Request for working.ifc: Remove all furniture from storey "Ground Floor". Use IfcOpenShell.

First a look at what the model holds.

```python
import ifcopenshell
import ifcopenshell.util.element

model = ifcopenshell.open("working.ifc")
print(model.schema)
storey = next(s for s in model.by_type("IfcBuildingStorey") if s.Name == "Ground Floor")
furniture = [e for e in ifcopenshell.util.element.get_decomposition(storey) if e.is_a("IfcFurnishingElement")]
seen = {}
for e in furniture:
    element_type = ifcopenshell.util.element.get_type(e)
    name = element_type.Name if element_type not in (None, e) else None
    seen[name] = seen.get(name, 0) + 1
for name, count in sorted(seen.items(), key=str):
    print(count, "x", name)
```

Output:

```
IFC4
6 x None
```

```python
import ifcopenshell
import ifcopenshell.api.root
import ifcopenshell.util.element

model = ifcopenshell.open("working.ifc")

storey = next(s for s in model.by_type("IfcBuildingStorey") if s.Name == "Ground Floor")
furniture = [e for e in ifcopenshell.util.element.get_decomposition(storey) if e.is_a("IfcFurnishingElement")]

for e in furniture:
    ifcopenshell.api.root.remove_product(model, product=e)
print(len(furniture), "removed")

model.write("working_edited.ifc")
```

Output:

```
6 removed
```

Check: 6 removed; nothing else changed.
